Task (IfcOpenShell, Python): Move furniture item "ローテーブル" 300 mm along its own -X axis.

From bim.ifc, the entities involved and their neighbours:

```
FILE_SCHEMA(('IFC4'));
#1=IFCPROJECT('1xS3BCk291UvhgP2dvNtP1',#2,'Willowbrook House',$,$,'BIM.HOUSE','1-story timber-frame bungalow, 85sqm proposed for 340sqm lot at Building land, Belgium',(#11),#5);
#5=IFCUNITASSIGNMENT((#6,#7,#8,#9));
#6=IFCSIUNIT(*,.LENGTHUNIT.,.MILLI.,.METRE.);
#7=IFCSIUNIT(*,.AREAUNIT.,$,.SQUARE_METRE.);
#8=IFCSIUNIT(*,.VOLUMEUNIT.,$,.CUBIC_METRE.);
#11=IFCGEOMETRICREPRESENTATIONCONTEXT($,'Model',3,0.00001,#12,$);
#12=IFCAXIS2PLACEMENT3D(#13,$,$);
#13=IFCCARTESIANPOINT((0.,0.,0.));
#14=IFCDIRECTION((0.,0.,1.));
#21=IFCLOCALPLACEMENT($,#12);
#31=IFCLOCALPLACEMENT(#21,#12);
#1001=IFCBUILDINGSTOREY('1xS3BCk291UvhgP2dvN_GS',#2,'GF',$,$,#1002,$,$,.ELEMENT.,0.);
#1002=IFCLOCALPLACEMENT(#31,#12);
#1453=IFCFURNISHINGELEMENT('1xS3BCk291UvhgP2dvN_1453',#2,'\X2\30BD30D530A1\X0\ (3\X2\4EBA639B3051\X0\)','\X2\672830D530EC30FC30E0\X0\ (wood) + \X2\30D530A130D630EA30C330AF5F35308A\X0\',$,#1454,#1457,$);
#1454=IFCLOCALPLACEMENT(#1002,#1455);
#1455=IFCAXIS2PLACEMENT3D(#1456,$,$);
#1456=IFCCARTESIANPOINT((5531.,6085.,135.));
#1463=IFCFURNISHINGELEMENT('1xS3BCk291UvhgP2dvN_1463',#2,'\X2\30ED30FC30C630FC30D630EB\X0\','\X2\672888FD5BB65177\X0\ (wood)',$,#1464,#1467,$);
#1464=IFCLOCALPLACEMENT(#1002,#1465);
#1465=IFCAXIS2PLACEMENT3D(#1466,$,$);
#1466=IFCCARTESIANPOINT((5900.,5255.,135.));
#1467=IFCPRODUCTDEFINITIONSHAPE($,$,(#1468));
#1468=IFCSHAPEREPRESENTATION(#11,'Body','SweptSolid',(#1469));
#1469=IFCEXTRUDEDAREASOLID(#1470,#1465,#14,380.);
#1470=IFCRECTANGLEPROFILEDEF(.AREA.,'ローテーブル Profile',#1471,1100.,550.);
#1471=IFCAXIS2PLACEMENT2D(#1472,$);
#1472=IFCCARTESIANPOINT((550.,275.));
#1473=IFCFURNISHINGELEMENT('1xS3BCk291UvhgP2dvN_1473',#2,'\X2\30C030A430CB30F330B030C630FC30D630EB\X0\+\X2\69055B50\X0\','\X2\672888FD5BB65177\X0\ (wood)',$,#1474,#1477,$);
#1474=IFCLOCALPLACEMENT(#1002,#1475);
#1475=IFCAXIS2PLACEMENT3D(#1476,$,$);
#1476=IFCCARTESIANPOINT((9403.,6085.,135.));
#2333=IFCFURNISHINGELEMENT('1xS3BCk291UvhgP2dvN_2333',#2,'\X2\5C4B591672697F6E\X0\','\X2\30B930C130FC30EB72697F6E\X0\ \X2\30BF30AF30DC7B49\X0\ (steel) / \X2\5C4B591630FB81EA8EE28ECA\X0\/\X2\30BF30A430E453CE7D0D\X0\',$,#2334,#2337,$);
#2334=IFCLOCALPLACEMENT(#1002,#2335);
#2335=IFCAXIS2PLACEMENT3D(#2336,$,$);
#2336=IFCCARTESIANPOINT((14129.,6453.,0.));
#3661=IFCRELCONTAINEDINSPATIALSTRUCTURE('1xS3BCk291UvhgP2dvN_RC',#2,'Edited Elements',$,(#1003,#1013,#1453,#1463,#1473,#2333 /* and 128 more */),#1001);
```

```python
import ifcopenshell
import ifcopenshell.api.geometry
import ifcopenshell.util.placement
import ifcopenshell.util.unit

model = ifcopenshell.open("bim.ifc")
unit_scale = ifcopenshell.util.unit.calculate_unit_scale(model)

item = model.by_guid("1xS3BCk291UvhgP2dvN_1463")
matrix = ifcopenshell.util.placement.get_local_placement(item.ObjectPlacement)
matrix[:3, 3] -= matrix[:3, 0] * 0.3 / unit_scale
ifcopenshell.api.geometry.edit_object_placement(model, product=item, matrix=matrix, is_si=False)

print(ifcopenshell.util.placement.get_local_placement(item.ObjectPlacement).round(3) + 0.0)

model.write("bim_v2.ifc")
```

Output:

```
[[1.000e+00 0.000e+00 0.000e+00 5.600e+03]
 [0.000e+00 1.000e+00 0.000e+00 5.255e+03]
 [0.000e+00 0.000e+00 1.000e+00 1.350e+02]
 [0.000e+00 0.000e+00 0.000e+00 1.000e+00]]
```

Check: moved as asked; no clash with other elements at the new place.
